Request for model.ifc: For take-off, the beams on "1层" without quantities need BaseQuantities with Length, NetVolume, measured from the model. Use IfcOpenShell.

First a look at what the model holds.

```python
import ifcopenshell
import ifcopenshell.util.element
import ifcopenshell.util.unit

model = ifcopenshell.open("model.ifc")
print(model.schema)
for unit_type in ("LENGTHUNIT", "AREAUNIT", "VOLUMEUNIT"):
    print(unit_type, ifcopenshell.util.unit.calculate_unit_scale(model, unit_type))
storey = next(s for s in model.by_type("IfcBuildingStorey") if s.Name == "1层")
beams = [e for e in ifcopenshell.util.element.get_decomposition(storey) if e.is_a("IfcBeam")]
for e in sorted(beams, key=lambda e: e.id()):
    print(e.id(), e.is_a(), e.Name, list(ifcopenshell.util.element.get_psets(e, qtos_only=True)), sep=" | ")
```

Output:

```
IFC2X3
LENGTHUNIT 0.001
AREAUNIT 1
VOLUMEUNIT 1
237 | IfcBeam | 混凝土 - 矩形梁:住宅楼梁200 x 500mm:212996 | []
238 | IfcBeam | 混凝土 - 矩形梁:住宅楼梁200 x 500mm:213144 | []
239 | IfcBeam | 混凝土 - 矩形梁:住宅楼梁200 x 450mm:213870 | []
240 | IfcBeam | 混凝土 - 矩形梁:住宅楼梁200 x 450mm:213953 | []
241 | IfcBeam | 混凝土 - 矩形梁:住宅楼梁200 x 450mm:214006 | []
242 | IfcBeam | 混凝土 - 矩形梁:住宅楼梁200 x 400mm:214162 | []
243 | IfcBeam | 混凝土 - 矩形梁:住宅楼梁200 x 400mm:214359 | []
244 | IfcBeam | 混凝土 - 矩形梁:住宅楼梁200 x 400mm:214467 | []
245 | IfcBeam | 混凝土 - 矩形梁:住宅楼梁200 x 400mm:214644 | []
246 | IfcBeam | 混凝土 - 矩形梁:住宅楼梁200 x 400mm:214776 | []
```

```python
import ifcopenshell
import ifcopenshell.api.pset
import ifcopenshell.geom
import ifcopenshell.util.element
import ifcopenshell.util.shape
import ifcopenshell.util.unit

model = ifcopenshell.open("model.ifc")
unit_scale = ifcopenshell.util.unit.calculate_unit_scale(model)
volume_scale = ifcopenshell.util.unit.calculate_unit_scale(model, "VOLUMEUNIT")
settings = ifcopenshell.geom.settings()

storey = next(s for s in model.by_type("IfcBuildingStorey") if s.Name == "1层")
beams = [e for e in ifcopenshell.util.element.get_decomposition(storey) if e.is_a("IfcBeam")]

for e in sorted(beams, key=lambda e: e.id()):
    if ifcopenshell.util.element.get_psets(e, qtos_only=True, should_inherit=False):
        continue
    # Geometry comes back in metres, in the element's own axes.
    shape = ifcopenshell.geom.create_shape(settings, e)
    values = {
        "Length": ifcopenshell.util.shape.get_max_xyz(shape.geometry) / unit_scale,
        "NetVolume": ifcopenshell.util.shape.get_volume(shape.geometry) / volume_scale,
    }
    qto = ifcopenshell.api.pset.add_qto(model, product=e, name="BaseQuantities")
    ifcopenshell.api.pset.edit_qto(model, qto=qto, properties=values)
    print(e.id(), {k: round(v, 3) for k, v in values.items()})

model.write("model_edited.ifc")
```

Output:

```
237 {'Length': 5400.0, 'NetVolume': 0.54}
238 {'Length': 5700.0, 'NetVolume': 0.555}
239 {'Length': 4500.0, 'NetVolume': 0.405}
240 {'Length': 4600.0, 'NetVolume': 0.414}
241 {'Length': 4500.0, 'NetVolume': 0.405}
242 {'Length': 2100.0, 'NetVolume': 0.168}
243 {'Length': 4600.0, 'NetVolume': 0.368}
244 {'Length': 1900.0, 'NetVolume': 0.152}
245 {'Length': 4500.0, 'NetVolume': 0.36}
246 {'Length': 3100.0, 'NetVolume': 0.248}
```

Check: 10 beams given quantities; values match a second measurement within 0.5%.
